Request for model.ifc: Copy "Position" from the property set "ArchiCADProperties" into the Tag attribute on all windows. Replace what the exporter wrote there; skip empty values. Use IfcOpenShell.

First a look at what the model holds.

```python
import ifcopenshell
import ifcopenshell.util.element

model = ifcopenshell.open("model.ifc")
print(model.schema)
windows = model.by_type("IfcWindow")
print(len(windows), "windows")
for e in windows[:8]:
    source = ifcopenshell.util.element.get_pset(e, "ArchiCADProperties", "Position")
    target = e.Tag
    print(e.id(), repr(source), repr(target), sep=" | ")
```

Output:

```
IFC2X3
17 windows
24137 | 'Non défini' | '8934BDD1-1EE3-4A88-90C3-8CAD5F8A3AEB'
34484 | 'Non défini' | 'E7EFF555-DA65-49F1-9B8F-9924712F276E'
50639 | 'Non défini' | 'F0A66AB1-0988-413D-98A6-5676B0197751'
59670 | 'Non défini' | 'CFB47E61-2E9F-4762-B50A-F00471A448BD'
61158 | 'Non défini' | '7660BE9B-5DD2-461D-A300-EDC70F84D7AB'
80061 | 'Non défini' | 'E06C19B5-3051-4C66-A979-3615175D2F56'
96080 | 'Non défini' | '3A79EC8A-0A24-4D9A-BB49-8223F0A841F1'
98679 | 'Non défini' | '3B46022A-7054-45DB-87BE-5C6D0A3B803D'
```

```python
import ifcopenshell
import ifcopenshell.util.element

model = ifcopenshell.open("model.ifc")

count = 0
for e in model.by_type("IfcWindow"):
    value = ifcopenshell.util.element.get_pset(e, "ArchiCADProperties", "Position")
    current = e.Tag
    if not value or not value.strip() or current == value:
        continue
    e.Tag = value
    count += 1

print(count, "windows updated")

model.write("model_edited.ifc")
```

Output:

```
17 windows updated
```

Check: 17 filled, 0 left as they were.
